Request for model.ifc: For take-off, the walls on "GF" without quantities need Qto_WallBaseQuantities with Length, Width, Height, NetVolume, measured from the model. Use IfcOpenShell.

First a look at what the model holds.

```python
import ifcopenshell
import ifcopenshell.util.element
import ifcopenshell.util.unit

model = ifcopenshell.open("model.ifc")
print(model.schema)
for unit_type in ("LENGTHUNIT", "AREAUNIT", "VOLUMEUNIT"):
    print(unit_type, ifcopenshell.util.unit.calculate_unit_scale(model, unit_type))
storey = next(s for s in model.by_type("IfcBuildingStorey") if s.Name == "GF")
walls = [e for e in ifcopenshell.util.element.get_decomposition(storey) if e.is_a("IfcWall")]
for e in sorted(walls, key=lambda e: e.id()):
    print(e.id(), e.is_a(), e.Name, list(ifcopenshell.util.element.get_psets(e, qtos_only=True)), sep=" | ")
```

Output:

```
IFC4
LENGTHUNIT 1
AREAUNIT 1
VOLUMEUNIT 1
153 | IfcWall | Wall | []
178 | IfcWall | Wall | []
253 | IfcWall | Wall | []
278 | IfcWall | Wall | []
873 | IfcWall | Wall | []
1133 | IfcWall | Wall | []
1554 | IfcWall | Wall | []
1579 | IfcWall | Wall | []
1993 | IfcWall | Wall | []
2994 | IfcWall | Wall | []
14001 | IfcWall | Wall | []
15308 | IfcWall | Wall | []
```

```python
import ifcopenshell
import ifcopenshell.api.pset
import ifcopenshell.geom
import ifcopenshell.util.element
import ifcopenshell.util.shape
import ifcopenshell.util.unit

model = ifcopenshell.open("model.ifc")
unit_scale = ifcopenshell.util.unit.calculate_unit_scale(model)
volume_scale = ifcopenshell.util.unit.calculate_unit_scale(model, "VOLUMEUNIT")
settings = ifcopenshell.geom.settings()

storey = next(s for s in model.by_type("IfcBuildingStorey") if s.Name == "GF")
walls = [e for e in ifcopenshell.util.element.get_decomposition(storey) if e.is_a("IfcWall")]

for e in sorted(walls, key=lambda e: e.id()):
    if ifcopenshell.util.element.get_psets(e, qtos_only=True, should_inherit=False):
        continue
    # Geometry comes back in metres, in the element's own axes.
    shape = ifcopenshell.geom.create_shape(settings, e)
    values = {
        "Length": ifcopenshell.util.shape.get_x(shape.geometry) / unit_scale,
        "Width": ifcopenshell.util.shape.get_y(shape.geometry) / unit_scale,
        "Height": ifcopenshell.util.shape.get_z(shape.geometry) / unit_scale,
        "NetVolume": ifcopenshell.util.shape.get_volume(shape.geometry) / volume_scale,
    }
    qto = ifcopenshell.api.pset.add_qto(model, product=e, name="Qto_WallBaseQuantities")
    ifcopenshell.api.pset.edit_qto(model, qto=qto, properties=values)
    print(e.id(), {k: round(v, 3) for k, v in values.items()})

model.write("model-out.ifc")
```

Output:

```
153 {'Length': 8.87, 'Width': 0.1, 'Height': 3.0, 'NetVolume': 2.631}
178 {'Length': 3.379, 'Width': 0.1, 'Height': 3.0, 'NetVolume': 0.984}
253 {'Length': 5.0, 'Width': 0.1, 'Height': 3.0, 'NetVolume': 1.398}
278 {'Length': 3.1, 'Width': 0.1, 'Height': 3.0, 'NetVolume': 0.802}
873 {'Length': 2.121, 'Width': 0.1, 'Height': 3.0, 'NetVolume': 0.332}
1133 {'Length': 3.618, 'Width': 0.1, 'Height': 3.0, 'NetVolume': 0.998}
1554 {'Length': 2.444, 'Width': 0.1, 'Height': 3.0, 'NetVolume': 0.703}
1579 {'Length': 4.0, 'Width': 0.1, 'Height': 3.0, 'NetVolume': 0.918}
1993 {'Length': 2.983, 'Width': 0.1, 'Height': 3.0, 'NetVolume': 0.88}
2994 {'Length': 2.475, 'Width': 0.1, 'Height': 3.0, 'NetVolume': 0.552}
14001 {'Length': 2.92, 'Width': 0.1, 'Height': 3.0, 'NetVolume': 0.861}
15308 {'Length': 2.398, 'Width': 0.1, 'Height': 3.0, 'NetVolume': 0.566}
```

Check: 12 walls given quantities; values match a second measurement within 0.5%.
